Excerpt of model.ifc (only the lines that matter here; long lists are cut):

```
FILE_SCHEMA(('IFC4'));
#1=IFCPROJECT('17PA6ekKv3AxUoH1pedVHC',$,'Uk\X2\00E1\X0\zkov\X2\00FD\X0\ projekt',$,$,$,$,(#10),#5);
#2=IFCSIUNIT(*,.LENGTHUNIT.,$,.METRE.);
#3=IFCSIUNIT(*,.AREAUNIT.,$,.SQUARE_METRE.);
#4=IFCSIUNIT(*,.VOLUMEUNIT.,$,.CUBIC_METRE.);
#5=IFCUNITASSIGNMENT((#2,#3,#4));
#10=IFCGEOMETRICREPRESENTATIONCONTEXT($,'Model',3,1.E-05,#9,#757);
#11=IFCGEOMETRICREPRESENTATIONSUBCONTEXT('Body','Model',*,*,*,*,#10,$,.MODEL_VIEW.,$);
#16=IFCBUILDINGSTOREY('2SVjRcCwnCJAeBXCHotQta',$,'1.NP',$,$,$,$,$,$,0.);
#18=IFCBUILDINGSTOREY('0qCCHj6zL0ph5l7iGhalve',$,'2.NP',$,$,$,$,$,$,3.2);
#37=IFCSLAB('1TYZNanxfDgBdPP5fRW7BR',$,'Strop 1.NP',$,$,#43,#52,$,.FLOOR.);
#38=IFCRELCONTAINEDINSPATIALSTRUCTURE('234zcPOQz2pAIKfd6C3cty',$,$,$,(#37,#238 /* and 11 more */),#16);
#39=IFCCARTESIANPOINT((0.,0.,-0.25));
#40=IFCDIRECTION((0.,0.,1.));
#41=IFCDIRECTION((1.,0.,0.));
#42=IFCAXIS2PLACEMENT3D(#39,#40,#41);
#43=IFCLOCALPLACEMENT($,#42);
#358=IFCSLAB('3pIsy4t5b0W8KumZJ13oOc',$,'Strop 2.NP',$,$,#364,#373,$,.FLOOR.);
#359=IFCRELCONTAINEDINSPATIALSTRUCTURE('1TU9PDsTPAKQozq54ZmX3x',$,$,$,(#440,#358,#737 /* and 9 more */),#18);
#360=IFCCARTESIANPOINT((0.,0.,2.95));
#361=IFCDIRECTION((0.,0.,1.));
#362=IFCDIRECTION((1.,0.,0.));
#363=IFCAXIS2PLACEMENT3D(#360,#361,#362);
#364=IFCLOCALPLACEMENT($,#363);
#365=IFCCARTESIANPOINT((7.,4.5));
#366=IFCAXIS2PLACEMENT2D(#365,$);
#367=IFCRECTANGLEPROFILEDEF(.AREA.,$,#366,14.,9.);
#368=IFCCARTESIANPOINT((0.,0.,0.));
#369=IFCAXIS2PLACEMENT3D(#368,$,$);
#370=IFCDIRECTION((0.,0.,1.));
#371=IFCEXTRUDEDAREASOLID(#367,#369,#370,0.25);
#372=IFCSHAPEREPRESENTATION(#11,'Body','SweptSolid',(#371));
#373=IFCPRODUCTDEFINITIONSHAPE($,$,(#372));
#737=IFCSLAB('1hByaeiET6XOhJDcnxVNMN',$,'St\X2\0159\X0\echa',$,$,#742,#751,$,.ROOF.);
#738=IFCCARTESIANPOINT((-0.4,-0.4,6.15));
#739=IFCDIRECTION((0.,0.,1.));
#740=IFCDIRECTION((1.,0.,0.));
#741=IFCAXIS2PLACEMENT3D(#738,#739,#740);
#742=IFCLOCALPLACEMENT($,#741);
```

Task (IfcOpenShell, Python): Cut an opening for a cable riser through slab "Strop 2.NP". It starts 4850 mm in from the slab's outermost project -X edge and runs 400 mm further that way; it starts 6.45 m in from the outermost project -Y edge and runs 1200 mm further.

```python
import numpy as np
import ifcopenshell
import ifcopenshell.api.feature
import ifcopenshell.api.geometry
import ifcopenshell.api.root
import ifcopenshell.geom
import ifcopenshell.util.placement
import ifcopenshell.util.representation
import ifcopenshell.util.shape
import ifcopenshell.util.unit

model = ifcopenshell.open("model.ifc")
unit_scale = ifcopenshell.util.unit.calculate_unit_scale(model)
settings = ifcopenshell.geom.settings()


def volume(element):
    """Net volume in cubic metres, openings subtracted."""
    shape = ifcopenshell.geom.create_shape(settings, element)
    return ifcopenshell.util.shape.get_volume(shape.geometry)


slab = model.by_guid("3pIsy4t5b0W8KumZJ13oOc")
before = volume(slab)

# Extent in the slab's own axes, in metres. The edges named are its -X and -Y sides.
slab_shape = ifcopenshell.geom.create_shape(settings, slab)
vertices = ifcopenshell.util.shape.get_vertices(slab_shape.geometry)
x_min, y_min, bottom = vertices.min(axis=0)
top = vertices[:, 2].max()

opening = ifcopenshell.api.root.create_entity(model, ifc_class="IfcOpeningElement", name="Cable riser opening", predefined_type="OPENING")
context = ifcopenshell.util.representation.get_context(model, "Model", "Body", "MODEL_VIEW")
width, depth = 0.4, 1.2
outline = [(0.0, 0.0), (width, 0.0), (width, depth), (0.0, depth), (0.0, 0.0)]
# Overshoot both faces by 50 mm so the cut is clean.
shape = ifcopenshell.api.geometry.add_slab_representation(
    model, context=context, depth=top - bottom + 0.1, polyline=outline
)
ifcopenshell.api.geometry.assign_representation(model, product=opening, representation=shape)

matrix = ifcopenshell.util.placement.get_local_placement(slab.ObjectPlacement)
matrix[:, 3] = matrix @ np.append(np.array([x_min + 4.85, y_min + 6.45, bottom - 0.05]) / unit_scale, 1.0)
ifcopenshell.api.geometry.edit_object_placement(model, product=opening, matrix=matrix, is_si=False)
ifcopenshell.api.feature.add_feature(model, feature=opening, element=slab)

after = volume(slab)

print(f"slab volume {before:.3f} -> {after:.3f} m3")

model.write("model_edited.ifc")
```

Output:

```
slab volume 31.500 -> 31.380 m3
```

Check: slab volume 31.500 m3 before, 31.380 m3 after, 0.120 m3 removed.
